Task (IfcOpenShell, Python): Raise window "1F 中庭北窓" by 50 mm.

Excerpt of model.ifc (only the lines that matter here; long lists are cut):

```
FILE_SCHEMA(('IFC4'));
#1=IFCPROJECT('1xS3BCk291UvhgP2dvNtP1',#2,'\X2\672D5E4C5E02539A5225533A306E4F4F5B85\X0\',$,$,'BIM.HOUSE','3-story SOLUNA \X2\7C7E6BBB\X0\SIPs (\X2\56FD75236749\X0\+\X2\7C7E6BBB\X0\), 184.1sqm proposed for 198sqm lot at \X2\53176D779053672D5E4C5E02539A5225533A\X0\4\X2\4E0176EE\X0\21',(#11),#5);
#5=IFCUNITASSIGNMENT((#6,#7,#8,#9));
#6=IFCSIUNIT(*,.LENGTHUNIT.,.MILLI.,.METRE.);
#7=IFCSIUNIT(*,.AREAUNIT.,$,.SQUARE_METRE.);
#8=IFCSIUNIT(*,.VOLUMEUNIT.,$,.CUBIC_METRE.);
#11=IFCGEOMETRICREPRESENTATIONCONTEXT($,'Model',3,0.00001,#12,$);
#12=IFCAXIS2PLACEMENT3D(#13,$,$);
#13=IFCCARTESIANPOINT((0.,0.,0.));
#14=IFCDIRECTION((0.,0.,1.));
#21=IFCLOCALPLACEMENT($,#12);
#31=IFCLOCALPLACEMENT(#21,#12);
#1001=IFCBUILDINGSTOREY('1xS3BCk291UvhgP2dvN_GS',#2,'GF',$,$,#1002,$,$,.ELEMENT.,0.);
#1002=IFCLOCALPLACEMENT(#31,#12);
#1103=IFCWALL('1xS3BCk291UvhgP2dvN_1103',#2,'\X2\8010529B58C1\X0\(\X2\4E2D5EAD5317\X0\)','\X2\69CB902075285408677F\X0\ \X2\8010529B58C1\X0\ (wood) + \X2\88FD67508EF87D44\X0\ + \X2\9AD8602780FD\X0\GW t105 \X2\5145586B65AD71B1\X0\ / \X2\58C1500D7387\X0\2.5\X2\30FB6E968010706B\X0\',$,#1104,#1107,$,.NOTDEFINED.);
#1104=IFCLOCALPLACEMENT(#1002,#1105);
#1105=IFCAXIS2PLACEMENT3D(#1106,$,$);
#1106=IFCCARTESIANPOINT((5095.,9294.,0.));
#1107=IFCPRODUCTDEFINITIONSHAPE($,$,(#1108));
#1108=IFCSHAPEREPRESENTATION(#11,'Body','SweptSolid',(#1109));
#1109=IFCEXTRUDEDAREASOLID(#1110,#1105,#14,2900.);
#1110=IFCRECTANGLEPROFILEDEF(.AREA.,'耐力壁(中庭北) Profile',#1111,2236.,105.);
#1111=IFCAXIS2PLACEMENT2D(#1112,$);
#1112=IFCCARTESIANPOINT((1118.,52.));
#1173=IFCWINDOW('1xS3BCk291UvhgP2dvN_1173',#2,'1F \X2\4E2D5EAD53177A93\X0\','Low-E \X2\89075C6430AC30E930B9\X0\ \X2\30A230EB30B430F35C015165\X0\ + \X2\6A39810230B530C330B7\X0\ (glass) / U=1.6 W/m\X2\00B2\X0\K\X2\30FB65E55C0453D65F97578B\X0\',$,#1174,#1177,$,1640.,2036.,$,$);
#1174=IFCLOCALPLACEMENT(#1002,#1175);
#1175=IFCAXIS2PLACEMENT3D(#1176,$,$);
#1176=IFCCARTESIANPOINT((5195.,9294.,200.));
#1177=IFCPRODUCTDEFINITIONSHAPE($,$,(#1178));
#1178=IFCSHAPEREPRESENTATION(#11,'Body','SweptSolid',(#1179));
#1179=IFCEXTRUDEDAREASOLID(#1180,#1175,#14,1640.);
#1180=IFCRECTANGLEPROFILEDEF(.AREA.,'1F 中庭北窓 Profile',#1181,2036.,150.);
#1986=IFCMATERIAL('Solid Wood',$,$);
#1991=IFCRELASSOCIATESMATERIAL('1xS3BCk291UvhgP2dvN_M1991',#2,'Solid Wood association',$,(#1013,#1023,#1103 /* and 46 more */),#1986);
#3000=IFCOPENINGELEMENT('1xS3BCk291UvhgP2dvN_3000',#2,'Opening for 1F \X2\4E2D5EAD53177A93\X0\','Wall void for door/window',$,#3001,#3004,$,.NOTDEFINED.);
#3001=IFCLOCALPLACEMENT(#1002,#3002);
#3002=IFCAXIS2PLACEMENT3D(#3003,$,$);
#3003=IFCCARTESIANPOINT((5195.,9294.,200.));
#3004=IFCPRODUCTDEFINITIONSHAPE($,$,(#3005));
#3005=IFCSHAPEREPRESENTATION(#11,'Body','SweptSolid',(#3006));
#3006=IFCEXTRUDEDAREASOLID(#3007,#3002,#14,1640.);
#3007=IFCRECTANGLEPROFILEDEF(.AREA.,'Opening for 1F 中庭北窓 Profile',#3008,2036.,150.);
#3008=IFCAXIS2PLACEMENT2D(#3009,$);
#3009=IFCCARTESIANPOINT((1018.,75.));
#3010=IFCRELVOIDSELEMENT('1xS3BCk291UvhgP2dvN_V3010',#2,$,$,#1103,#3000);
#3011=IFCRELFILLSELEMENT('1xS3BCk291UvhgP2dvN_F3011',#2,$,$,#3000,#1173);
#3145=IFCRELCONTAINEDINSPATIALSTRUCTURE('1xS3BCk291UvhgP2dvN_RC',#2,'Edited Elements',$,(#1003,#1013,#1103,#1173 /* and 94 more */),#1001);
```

```python
import numpy as np
import ifcopenshell
import ifcopenshell.api.geometry
import ifcopenshell.util.placement
import ifcopenshell.util.unit

model = ifcopenshell.open("model.ifc")
unit_scale = ifcopenshell.util.unit.calculate_unit_scale(model)

window = model.by_guid("1xS3BCk291UvhgP2dvN_1173")
opening = window.FillsVoids[0].RelatingOpeningElement
dz = 0.05 / unit_scale

shift = np.array([0.0, 0.0, dz])
# The window is not placed relative to its opening, so move both.
for product in (opening, window):
    matrix = ifcopenshell.util.placement.get_local_placement(product.ObjectPlacement)
    matrix[:3, 3] += shift
    ifcopenshell.api.geometry.edit_object_placement(model, product=product, matrix=matrix, is_si=False)

print(f"moved by {dz * unit_scale:+.3f} m")

model.write("model_updated.ifc")
```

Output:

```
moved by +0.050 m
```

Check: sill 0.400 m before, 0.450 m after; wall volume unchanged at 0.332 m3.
